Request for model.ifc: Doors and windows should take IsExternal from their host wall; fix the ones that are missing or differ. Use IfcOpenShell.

First a look at what the model holds.

```python
import ifcopenshell
import ifcopenshell.util.element

model = ifcopenshell.open("model.ifc")
print(model.schema)
seen = {}
for e in model.by_type("IfcDoor") + model.by_type("IfcWindow"):
    if not e.FillsVoids:
        continue
    host = e.FillsVoids[0].RelatingOpeningElement.VoidsElements[0].RelatingBuildingElement
    own = ifcopenshell.util.element.get_pset(e, f"Pset_{e.is_a()[3:].removesuffix('StandardCase')}Common", "IsExternal")
    wall = ifcopenshell.util.element.get_pset(host, "Pset_WallCommon", "IsExternal")
    seen[e.is_a(), own, wall] = seen.get((e.is_a(), own, wall), 0) + 1
for (cls, own, wall), count in sorted(seen.items(), key=str):
    print(count, cls, "IsExternal:", own, "| host wall:", wall)
```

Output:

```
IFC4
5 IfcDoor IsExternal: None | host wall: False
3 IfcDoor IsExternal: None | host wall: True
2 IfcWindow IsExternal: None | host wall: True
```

```python
import ifcopenshell
import ifcopenshell.api.pset
import ifcopenshell.util.element

model = ifcopenshell.open("model.ifc")

count = 0
for ifc_class, pset_name in (("IfcDoor", "Pset_DoorCommon"), ("IfcWindow", "Pset_WindowCommon")):
    for e in model.by_type(ifc_class):
        if not e.FillsVoids:
            continue
        host = e.FillsVoids[0].RelatingOpeningElement.VoidsElements[0].RelatingBuildingElement
        external = ifcopenshell.util.element.get_pset(host, "Pset_WallCommon", "IsExternal")
        if external is None or ifcopenshell.util.element.get_pset(e, pset_name, "IsExternal") == external:
            continue
        pset = ifcopenshell.api.pset.add_pset(model, product=e, name=pset_name)
        ifcopenshell.api.pset.edit_pset(model, pset=pset, properties={"IsExternal": external})
        count += 1

print(count, "updated")

model.write("model_rev.ifc")
```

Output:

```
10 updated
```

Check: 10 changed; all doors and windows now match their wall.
